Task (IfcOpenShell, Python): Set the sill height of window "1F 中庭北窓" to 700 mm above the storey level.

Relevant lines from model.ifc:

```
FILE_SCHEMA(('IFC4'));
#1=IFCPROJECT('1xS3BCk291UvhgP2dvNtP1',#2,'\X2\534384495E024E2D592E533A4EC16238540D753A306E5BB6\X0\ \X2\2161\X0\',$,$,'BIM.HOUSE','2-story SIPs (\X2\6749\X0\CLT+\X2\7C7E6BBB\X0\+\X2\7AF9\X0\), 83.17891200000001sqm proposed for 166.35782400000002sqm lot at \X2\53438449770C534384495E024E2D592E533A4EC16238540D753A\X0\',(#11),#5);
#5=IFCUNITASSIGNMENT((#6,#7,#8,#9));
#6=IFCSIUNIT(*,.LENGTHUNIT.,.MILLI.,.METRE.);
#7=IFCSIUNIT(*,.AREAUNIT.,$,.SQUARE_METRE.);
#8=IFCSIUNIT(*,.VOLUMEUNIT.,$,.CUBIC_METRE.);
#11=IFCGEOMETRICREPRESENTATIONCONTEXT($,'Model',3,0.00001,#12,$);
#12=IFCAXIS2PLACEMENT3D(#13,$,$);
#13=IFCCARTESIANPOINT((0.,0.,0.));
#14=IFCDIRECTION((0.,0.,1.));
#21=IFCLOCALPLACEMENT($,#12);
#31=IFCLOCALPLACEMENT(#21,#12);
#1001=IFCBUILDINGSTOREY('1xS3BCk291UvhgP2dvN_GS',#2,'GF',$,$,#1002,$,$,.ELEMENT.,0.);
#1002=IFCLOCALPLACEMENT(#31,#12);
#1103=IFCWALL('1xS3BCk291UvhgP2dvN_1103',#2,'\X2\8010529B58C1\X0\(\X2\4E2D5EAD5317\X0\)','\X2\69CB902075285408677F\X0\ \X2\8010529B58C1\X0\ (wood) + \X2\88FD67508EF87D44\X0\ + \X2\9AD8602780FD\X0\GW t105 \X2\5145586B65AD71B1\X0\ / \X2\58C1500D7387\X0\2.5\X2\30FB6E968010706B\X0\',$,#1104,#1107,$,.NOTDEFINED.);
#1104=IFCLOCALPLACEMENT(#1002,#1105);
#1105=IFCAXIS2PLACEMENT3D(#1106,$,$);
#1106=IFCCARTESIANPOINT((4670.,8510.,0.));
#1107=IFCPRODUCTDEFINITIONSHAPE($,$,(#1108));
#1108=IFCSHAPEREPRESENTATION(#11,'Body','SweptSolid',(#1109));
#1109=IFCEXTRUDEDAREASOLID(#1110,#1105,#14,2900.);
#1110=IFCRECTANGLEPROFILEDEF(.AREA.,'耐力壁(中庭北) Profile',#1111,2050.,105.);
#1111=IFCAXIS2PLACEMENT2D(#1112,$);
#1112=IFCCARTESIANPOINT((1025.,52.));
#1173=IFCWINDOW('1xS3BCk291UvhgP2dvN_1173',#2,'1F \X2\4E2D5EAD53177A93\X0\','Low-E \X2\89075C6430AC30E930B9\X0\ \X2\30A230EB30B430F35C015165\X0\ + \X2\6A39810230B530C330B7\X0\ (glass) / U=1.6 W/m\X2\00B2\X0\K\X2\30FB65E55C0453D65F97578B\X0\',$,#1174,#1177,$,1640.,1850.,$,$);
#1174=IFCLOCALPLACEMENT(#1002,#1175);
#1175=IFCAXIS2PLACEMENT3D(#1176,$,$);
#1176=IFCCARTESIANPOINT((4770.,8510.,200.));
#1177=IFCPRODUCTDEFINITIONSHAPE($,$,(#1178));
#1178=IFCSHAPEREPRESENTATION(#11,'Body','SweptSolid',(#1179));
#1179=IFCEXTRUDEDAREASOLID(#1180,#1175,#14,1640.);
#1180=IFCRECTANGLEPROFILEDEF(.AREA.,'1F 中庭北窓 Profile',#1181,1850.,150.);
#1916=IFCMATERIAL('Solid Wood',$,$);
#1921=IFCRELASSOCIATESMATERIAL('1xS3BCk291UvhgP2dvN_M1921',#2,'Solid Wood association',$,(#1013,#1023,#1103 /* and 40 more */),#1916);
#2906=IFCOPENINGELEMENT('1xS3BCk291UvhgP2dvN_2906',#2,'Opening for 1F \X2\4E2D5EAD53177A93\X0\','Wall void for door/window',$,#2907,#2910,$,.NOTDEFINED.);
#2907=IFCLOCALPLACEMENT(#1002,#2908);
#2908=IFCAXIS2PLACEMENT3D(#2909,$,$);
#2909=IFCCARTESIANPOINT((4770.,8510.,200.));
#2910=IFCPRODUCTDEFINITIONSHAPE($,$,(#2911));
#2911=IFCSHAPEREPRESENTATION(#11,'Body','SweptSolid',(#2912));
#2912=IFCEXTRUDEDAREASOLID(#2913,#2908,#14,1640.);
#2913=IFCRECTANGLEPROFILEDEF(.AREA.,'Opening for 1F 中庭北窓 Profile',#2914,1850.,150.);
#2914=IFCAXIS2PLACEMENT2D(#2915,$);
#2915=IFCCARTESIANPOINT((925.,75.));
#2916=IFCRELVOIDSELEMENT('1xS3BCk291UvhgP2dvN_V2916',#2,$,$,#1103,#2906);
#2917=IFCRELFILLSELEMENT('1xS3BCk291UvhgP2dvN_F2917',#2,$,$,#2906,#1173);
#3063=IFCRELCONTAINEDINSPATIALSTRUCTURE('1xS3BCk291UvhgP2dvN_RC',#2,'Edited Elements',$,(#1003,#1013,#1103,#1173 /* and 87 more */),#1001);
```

```python
import numpy as np
import ifcopenshell
import ifcopenshell.api.geometry
import ifcopenshell.geom
import ifcopenshell.util.element
import ifcopenshell.util.placement
import ifcopenshell.util.shape
import ifcopenshell.util.unit

model = ifcopenshell.open("model.ifc")
unit_scale = ifcopenshell.util.unit.calculate_unit_scale(model)

window = model.by_guid("1xS3BCk291UvhgP2dvN_1173")
opening = window.FillsVoids[0].RelatingOpeningElement
storey = ifcopenshell.util.element.get_container(window, ifc_class="IfcBuildingStorey")
level = ifcopenshell.util.placement.get_local_placement(storey.ObjectPlacement)[2, 3]

# The opening's origin need not be at the sill, so measure its lowest point.
shape = ifcopenshell.geom.create_shape(ifcopenshell.geom.settings(), opening)
bottom = ifcopenshell.util.shape.get_shape_bottom_elevation(shape, shape.geometry) / unit_scale
dz = level + 0.7 / unit_scale - bottom

shift = np.array([0.0, 0.0, dz])
# The window is not placed relative to its opening, so move both.
for product in (opening, window):
    matrix = ifcopenshell.util.placement.get_local_placement(product.ObjectPlacement)
    matrix[:3, 3] += shift
    ifcopenshell.api.geometry.edit_object_placement(model, product=product, matrix=matrix, is_si=False)

print(f"moved by {dz * unit_scale:+.3f} m")

model.write("model_edited.ifc")
```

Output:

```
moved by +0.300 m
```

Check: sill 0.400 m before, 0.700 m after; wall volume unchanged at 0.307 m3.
